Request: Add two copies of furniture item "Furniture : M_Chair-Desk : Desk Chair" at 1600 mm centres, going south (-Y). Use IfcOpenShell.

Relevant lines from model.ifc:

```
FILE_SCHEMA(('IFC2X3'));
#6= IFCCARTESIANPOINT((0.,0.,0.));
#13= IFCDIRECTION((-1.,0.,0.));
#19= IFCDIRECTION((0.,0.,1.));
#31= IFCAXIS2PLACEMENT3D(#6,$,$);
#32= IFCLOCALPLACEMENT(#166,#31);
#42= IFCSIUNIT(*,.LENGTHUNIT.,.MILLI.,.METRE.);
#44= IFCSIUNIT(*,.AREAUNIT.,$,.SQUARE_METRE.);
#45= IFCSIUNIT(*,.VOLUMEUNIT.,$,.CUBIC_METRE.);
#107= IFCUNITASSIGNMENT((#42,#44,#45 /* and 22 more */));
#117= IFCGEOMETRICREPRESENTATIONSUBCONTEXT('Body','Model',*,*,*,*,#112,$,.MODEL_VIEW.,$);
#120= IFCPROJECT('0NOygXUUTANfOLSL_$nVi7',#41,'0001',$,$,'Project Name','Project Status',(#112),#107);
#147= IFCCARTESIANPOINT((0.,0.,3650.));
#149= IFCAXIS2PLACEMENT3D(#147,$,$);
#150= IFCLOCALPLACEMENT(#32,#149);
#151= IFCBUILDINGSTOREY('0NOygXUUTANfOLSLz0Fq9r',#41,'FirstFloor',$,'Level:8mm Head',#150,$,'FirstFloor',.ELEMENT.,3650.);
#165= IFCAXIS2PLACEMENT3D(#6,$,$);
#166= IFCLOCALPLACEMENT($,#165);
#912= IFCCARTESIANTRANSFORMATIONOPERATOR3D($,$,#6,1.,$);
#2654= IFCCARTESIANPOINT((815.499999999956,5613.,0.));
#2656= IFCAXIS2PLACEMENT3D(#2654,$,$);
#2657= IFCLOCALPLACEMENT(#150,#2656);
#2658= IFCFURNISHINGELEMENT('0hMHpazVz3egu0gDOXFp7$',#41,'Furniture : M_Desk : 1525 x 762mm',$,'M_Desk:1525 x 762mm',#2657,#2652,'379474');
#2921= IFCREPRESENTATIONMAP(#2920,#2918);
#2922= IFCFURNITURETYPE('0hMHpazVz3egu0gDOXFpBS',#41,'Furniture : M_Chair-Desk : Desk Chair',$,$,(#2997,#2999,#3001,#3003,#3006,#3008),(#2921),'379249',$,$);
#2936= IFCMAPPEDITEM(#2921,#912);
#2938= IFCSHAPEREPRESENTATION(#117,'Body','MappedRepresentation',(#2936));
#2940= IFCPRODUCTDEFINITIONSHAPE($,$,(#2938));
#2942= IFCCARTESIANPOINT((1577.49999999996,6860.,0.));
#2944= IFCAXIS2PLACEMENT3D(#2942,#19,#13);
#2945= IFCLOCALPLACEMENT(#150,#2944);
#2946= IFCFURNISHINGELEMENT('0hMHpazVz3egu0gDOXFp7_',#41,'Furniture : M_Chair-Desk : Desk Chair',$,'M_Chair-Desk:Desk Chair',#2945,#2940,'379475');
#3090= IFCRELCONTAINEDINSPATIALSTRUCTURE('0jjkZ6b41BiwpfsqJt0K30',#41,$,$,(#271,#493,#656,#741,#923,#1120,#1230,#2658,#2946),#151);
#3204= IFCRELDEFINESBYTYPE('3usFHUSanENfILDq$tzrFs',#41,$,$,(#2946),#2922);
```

```python
import numpy as np
import ifcopenshell
import ifcopenshell.api.geometry
import ifcopenshell.api.root
import ifcopenshell.util.element
import ifcopenshell.util.placement
import ifcopenshell.util.unit

model = ifcopenshell.open("model.ifc")
unit_scale = ifcopenshell.util.unit.calculate_unit_scale(model)


def reuse_history(source, copy):
    """copy_class also copies each property set's owner history, people and application; keep the originals."""
    for rel in copy.IsDefinedBy:
        if rel.is_a("IfcRelDefinesByProperties") and (history := rel.RelatingPropertyDefinition.OwnerHistory):
            rel.RelatingPropertyDefinition.OwnerHistory = source.OwnerHistory
            ifcopenshell.util.element.remove_deep2(model, history)


source = model.by_id(2946)
base = ifcopenshell.util.placement.get_local_placement(source.ObjectPlacement)
step = np.array([0.0, -1.0, 0.0]) * 1.6 / unit_scale

for i in range(1, 3):
    copy = ifcopenshell.api.root.copy_class(model, product=source)
    copy.Representation = ifcopenshell.util.element.copy_deep(
        model, source.Representation, exclude=["IfcGeometricRepresentationContext", "IfcRepresentationMap"]
    )
    copy.Tag = None
    reuse_history(source, copy)
    matrix = base.copy()
    matrix[:3, 3] += i * step
    print("added at", matrix[:3, 3].round(3) + 0.0)
    ifcopenshell.api.geometry.edit_object_placement(model, product=copy, matrix=matrix, is_si=False)

model.write("model_edited.ifc")
```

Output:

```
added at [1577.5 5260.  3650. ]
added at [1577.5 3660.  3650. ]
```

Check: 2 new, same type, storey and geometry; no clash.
